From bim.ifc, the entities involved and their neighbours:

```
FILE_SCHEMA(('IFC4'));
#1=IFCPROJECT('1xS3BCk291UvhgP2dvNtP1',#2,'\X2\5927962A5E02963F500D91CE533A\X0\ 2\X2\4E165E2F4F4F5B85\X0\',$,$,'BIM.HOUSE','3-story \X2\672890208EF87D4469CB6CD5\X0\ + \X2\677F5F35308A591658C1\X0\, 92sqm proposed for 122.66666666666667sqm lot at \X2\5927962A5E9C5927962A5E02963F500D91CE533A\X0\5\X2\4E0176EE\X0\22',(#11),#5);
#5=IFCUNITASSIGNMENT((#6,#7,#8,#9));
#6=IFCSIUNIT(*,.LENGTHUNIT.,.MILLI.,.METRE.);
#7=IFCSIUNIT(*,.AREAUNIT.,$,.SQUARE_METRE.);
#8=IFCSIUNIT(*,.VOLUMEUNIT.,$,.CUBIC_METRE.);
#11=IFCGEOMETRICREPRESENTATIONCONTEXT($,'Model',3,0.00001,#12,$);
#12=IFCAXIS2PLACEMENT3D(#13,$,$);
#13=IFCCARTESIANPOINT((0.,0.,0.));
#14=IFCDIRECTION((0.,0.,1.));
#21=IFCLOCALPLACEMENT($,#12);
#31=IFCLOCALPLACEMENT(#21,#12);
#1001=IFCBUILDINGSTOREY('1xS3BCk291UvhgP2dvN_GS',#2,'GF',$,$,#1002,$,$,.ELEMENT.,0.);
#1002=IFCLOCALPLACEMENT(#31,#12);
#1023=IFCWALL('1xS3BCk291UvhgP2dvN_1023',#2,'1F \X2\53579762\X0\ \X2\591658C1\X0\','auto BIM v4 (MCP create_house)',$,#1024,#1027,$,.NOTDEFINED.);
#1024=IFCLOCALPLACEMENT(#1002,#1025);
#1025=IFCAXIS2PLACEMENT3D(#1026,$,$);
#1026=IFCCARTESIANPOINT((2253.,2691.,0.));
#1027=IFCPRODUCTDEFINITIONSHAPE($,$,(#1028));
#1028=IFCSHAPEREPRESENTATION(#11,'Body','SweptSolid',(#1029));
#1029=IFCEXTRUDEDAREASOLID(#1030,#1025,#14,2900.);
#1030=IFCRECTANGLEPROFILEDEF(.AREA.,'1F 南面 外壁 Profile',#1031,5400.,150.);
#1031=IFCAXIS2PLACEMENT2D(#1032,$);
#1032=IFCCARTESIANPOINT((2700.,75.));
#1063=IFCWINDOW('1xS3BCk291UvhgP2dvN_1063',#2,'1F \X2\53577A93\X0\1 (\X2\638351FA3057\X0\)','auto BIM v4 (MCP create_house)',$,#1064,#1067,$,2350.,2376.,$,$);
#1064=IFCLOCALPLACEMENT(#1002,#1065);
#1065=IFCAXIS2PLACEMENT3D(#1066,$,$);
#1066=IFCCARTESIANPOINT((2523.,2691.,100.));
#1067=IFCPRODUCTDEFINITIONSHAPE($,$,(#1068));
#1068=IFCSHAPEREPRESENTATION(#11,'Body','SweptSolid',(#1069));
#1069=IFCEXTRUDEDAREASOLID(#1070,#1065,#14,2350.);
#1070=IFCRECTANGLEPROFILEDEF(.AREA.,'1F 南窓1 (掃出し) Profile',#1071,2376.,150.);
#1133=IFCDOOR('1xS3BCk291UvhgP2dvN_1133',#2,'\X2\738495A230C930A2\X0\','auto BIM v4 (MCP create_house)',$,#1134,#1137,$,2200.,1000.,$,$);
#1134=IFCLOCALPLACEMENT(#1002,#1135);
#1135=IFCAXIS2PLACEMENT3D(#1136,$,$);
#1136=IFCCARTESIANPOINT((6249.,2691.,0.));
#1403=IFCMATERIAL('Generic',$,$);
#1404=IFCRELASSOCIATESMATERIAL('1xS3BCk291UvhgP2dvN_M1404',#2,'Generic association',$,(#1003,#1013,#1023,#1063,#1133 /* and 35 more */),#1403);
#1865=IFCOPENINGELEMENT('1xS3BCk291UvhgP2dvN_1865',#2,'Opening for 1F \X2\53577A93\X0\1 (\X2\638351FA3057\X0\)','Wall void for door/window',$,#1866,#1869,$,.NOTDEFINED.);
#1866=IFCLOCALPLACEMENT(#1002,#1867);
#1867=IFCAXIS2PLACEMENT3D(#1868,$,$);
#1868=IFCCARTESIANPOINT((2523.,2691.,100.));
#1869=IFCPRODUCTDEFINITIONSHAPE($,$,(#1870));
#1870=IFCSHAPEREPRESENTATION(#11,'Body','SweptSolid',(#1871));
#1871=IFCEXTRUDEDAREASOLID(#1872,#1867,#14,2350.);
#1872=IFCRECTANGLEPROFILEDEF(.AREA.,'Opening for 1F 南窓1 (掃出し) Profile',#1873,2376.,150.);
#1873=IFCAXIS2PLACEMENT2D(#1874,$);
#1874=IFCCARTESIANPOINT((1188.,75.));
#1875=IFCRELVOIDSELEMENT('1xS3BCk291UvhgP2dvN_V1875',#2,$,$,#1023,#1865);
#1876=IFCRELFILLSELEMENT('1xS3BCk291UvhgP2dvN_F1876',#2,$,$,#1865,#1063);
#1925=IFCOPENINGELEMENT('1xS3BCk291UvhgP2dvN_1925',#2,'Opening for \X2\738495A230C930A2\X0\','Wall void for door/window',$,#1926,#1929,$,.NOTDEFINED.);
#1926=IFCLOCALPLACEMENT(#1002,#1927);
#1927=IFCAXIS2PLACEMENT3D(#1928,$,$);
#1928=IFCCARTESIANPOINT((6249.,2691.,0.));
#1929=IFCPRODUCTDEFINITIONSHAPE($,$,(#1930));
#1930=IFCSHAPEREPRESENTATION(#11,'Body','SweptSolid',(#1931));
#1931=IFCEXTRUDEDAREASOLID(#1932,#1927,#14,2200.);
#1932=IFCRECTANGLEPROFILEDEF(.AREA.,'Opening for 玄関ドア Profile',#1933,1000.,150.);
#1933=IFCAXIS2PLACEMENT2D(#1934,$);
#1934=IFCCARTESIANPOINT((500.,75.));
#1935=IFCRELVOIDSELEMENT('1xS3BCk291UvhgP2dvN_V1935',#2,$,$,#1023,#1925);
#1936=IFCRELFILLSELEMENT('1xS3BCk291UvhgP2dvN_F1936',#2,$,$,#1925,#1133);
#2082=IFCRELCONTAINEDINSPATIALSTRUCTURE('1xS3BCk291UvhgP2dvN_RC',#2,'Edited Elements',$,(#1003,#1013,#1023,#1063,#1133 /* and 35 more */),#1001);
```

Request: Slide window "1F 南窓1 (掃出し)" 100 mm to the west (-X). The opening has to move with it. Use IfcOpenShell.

```python
import ifcopenshell
import ifcopenshell.api.geometry
import ifcopenshell.util.placement

model = ifcopenshell.open("bim.ifc")

window = model.by_guid("1xS3BCk291UvhgP2dvN_1063")
opening = window.FillsVoids[0].RelatingOpeningElement
wall = opening.VoidsElements[0].RelatingBuildingElement

wall_matrix = ifcopenshell.util.placement.get_local_placement(wall.ObjectPlacement)
shift = wall_matrix[:3, 0] * -100.0
before = ifcopenshell.util.placement.get_local_placement(window.ObjectPlacement)[:3, 3].copy()

# The window is not placed relative to its opening, so move both.
for product in (opening, window):
    matrix = ifcopenshell.util.placement.get_local_placement(product.ObjectPlacement)
    matrix[:3, 3] += shift
    ifcopenshell.api.geometry.edit_object_placement(model, product=product, matrix=matrix, is_si=False)

after = ifcopenshell.util.placement.get_local_placement(window.ObjectPlacement)[:3, 3]
print("window moved by", (after - before).round(3) + 0.0)

model.write("bim_rev.ifc")
```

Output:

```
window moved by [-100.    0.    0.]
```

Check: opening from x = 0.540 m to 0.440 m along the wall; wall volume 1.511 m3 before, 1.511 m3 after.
